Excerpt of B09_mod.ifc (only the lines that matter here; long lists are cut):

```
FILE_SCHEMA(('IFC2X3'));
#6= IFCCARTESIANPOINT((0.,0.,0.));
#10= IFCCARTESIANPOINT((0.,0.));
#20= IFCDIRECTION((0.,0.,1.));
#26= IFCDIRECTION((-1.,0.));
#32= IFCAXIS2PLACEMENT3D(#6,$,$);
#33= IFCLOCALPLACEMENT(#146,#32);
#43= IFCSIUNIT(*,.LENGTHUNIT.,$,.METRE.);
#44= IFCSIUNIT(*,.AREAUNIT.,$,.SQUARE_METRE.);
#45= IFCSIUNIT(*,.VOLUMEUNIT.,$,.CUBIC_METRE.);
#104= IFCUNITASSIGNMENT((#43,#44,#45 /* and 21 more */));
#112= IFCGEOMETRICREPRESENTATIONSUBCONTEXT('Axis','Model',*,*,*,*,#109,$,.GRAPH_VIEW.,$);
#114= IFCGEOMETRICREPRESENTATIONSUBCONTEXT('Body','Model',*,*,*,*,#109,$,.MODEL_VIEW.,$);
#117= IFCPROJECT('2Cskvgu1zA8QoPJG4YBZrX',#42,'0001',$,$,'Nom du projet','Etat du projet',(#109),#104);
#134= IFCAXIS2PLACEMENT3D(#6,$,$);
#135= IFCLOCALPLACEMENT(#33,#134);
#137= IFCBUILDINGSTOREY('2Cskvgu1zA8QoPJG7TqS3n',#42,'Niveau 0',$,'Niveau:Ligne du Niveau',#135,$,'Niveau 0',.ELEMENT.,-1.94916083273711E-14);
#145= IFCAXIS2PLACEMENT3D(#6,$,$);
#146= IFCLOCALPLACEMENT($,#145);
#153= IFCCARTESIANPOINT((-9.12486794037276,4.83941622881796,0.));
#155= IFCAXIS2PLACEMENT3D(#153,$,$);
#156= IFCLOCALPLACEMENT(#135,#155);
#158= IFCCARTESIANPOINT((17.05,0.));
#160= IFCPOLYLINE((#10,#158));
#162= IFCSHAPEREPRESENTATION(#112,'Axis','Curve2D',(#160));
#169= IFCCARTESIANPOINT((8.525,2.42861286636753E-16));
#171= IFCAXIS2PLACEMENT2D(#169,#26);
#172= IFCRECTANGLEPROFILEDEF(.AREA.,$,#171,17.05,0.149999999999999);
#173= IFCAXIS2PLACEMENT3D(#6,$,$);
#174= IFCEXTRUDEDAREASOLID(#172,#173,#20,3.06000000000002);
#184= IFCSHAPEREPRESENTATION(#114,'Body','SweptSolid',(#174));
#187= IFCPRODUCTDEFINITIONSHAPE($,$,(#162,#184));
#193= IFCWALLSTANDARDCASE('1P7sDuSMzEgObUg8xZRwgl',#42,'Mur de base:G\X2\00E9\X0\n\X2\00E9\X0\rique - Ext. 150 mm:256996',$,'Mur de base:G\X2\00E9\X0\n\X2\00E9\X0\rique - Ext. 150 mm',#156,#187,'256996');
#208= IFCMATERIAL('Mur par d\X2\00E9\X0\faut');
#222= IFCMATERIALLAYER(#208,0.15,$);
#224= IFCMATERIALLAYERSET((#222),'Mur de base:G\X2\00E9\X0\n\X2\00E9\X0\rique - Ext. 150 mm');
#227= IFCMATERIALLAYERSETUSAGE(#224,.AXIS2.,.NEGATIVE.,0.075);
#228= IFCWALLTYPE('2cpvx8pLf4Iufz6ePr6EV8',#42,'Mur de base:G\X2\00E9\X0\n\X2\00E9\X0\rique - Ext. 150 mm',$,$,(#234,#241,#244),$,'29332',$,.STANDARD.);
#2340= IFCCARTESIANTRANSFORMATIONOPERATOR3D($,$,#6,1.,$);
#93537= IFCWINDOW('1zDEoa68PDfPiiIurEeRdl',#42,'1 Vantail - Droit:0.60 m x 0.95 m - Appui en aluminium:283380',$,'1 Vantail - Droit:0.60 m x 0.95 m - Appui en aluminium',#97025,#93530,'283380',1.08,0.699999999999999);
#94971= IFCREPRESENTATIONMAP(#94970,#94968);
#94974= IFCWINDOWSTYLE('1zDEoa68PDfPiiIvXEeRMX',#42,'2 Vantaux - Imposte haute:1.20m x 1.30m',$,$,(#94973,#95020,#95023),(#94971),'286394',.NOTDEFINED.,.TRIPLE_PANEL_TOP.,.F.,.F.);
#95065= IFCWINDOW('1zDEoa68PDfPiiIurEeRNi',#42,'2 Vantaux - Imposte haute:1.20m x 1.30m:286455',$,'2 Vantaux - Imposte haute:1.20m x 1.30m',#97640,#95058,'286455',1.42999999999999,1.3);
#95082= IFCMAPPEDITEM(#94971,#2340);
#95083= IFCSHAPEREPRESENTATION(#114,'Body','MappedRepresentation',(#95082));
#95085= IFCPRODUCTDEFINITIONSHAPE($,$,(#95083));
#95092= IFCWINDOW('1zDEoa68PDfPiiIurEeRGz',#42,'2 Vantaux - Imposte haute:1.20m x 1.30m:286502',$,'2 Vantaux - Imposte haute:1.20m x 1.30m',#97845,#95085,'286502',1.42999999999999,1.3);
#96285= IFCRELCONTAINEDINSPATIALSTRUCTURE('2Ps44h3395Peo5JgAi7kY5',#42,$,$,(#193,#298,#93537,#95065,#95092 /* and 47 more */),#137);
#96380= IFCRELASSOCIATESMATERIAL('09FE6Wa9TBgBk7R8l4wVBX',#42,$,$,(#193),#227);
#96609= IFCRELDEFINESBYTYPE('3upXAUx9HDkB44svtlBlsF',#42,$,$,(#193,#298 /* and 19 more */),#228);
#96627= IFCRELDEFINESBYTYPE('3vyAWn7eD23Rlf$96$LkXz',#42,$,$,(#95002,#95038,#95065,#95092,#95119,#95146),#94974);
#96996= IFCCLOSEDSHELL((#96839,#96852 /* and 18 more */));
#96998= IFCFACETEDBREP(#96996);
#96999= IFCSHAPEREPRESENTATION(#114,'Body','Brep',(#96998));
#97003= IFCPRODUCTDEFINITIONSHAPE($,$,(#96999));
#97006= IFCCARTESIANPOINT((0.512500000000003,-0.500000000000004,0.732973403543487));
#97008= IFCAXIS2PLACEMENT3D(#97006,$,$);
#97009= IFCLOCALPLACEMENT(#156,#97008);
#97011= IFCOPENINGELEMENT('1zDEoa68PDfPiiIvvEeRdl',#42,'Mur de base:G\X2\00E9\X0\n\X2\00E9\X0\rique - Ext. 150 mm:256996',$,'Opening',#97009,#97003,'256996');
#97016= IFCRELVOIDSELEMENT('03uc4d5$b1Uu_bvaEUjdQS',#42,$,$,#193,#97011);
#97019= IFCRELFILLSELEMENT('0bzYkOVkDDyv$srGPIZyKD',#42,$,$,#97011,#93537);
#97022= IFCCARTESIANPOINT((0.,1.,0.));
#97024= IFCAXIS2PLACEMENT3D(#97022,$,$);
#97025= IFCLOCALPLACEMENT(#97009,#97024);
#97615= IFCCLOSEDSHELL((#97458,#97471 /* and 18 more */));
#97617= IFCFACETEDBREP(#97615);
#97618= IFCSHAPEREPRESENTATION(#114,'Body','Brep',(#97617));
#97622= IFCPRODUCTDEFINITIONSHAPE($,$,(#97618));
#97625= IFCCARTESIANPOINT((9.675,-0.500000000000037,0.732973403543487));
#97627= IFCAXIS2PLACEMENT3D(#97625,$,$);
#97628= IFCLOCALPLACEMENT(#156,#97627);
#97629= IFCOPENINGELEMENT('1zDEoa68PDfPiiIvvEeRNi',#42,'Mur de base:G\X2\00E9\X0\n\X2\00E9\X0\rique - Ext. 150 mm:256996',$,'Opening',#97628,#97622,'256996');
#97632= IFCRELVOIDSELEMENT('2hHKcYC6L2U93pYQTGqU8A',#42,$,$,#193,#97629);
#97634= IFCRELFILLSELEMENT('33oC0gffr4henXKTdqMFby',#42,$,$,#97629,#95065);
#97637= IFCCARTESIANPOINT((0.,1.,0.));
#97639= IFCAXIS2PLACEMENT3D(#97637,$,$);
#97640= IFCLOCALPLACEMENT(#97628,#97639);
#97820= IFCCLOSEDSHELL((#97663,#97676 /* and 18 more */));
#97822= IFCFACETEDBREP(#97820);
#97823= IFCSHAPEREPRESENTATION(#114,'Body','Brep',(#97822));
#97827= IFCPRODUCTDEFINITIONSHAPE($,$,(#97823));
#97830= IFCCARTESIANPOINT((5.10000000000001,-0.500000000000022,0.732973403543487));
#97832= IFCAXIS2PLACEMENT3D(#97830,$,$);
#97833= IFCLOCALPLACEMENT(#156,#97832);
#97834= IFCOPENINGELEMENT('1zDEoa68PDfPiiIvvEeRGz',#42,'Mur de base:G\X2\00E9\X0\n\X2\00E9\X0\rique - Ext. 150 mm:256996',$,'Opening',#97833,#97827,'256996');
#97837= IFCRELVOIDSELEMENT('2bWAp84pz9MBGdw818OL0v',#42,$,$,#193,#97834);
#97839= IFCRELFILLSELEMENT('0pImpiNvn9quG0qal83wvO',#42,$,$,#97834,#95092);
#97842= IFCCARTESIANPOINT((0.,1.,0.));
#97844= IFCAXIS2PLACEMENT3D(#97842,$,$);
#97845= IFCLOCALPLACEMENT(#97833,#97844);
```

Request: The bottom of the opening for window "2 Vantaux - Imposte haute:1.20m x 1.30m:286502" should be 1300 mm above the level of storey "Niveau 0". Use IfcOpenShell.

```python
import numpy as np
import ifcopenshell
import ifcopenshell.api.geometry
import ifcopenshell.geom
import ifcopenshell.util.element
import ifcopenshell.util.placement
import ifcopenshell.util.shape
import ifcopenshell.util.unit

model = ifcopenshell.open("B09_mod.ifc")
unit_scale = ifcopenshell.util.unit.calculate_unit_scale(model)

window = model.by_guid("1zDEoa68PDfPiiIurEeRGz")
opening = window.FillsVoids[0].RelatingOpeningElement
storey = ifcopenshell.util.element.get_container(window, ifc_class="IfcBuildingStorey")
level = ifcopenshell.util.placement.get_local_placement(storey.ObjectPlacement)[2, 3]

# The opening's origin need not be at the sill, so measure its lowest point.
shape = ifcopenshell.geom.create_shape(ifcopenshell.geom.settings(), opening)
bottom = ifcopenshell.util.shape.get_shape_bottom_elevation(shape, shape.geometry) / unit_scale
dz = level + 1.3 - bottom

shift = np.array([0.0, 0.0, dz])
# The window is placed relative to its opening, so it follows when the opening moves.
matrix = ifcopenshell.util.placement.get_local_placement(opening.ObjectPlacement)
matrix[:3, 3] += shift
ifcopenshell.api.geometry.edit_object_placement(
    model, product=opening, matrix=matrix, is_si=False, should_transform_children=True
)

print(f"moved by {dz * unit_scale:+.3f} m")

model.write("B09_mod-out.ifc")
```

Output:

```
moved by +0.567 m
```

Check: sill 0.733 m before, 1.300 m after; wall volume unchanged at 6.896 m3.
